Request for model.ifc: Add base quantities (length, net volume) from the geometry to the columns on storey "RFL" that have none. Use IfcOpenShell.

First a look at what the model holds.

```python
import ifcopenshell
import ifcopenshell.util.element
import ifcopenshell.util.unit

model = ifcopenshell.open("model.ifc")
print(model.schema)
for unit_type in ("LENGTHUNIT", "AREAUNIT", "VOLUMEUNIT"):
    print(unit_type, ifcopenshell.util.unit.calculate_unit_scale(model, unit_type))
storey = next(s for s in model.by_type("IfcBuildingStorey") if s.Name == "RFL")
columns = [e for e in ifcopenshell.util.element.get_decomposition(storey) if e.is_a("IfcColumn")]
for e in sorted(columns, key=lambda e: e.id()):
    print(e.id(), e.is_a(), e.Name, list(ifcopenshell.util.element.get_psets(e, qtos_only=True)), sep=" | ")
```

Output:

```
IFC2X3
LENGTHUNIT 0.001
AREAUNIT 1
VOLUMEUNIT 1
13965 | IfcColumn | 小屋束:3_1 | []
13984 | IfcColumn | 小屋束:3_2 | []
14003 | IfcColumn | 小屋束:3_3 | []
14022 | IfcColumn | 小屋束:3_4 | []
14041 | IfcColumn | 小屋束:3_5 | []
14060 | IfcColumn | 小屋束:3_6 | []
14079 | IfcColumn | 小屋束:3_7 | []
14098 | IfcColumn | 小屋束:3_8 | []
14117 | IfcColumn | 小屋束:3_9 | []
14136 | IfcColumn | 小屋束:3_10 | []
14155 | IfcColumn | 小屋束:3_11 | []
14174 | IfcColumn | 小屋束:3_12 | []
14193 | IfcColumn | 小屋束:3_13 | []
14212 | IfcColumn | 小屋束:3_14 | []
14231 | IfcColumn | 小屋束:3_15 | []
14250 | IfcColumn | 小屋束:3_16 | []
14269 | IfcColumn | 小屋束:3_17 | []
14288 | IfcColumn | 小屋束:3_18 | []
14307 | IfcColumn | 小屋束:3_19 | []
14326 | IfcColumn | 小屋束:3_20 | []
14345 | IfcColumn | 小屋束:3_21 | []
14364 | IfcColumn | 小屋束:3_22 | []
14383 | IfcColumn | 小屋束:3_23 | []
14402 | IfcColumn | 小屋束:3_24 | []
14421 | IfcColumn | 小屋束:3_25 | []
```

```python
import ifcopenshell
import ifcopenshell.api.pset
import ifcopenshell.geom
import ifcopenshell.util.element
import ifcopenshell.util.shape
import ifcopenshell.util.unit

model = ifcopenshell.open("model.ifc")
unit_scale = ifcopenshell.util.unit.calculate_unit_scale(model)
volume_scale = ifcopenshell.util.unit.calculate_unit_scale(model, "VOLUMEUNIT")
settings = ifcopenshell.geom.settings()

storey = next(s for s in model.by_type("IfcBuildingStorey") if s.Name == "RFL")
columns = [e for e in ifcopenshell.util.element.get_decomposition(storey) if e.is_a("IfcColumn")]

for e in sorted(columns, key=lambda e: e.id()):
    if ifcopenshell.util.element.get_psets(e, qtos_only=True, should_inherit=False):
        continue
    # Geometry comes back in metres, in the element's own axes.
    shape = ifcopenshell.geom.create_shape(settings, e)
    values = {
        "Length": ifcopenshell.util.shape.get_z(shape.geometry) / unit_scale,
        "NetVolume": ifcopenshell.util.shape.get_volume(shape.geometry) / volume_scale,
    }
    qto = ifcopenshell.api.pset.add_qto(model, product=e, name="BaseQuantities")
    ifcopenshell.api.pset.edit_qto(model, qto=qto, properties=values)
    print(e.id(), {k: round(v, 3) for k, v in values.items()})

model.write("model_edited.ifc")
```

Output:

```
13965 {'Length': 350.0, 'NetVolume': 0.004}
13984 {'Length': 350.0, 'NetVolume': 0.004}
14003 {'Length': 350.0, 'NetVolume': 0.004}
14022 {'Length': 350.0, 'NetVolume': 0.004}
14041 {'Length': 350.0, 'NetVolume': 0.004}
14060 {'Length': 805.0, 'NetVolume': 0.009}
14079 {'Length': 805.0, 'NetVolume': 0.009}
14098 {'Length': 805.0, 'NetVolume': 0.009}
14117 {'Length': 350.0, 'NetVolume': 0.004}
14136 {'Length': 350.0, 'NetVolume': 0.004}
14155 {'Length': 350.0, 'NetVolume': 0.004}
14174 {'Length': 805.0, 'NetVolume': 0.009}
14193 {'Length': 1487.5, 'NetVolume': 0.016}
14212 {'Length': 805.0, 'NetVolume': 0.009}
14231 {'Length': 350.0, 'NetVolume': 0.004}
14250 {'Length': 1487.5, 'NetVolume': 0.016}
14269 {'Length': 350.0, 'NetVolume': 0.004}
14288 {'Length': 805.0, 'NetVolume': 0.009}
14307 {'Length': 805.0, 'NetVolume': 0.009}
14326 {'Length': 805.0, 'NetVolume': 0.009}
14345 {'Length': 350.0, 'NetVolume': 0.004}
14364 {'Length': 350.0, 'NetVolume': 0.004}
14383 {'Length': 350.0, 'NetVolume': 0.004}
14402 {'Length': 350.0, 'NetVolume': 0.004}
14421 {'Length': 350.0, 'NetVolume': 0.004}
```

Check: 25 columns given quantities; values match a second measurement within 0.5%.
